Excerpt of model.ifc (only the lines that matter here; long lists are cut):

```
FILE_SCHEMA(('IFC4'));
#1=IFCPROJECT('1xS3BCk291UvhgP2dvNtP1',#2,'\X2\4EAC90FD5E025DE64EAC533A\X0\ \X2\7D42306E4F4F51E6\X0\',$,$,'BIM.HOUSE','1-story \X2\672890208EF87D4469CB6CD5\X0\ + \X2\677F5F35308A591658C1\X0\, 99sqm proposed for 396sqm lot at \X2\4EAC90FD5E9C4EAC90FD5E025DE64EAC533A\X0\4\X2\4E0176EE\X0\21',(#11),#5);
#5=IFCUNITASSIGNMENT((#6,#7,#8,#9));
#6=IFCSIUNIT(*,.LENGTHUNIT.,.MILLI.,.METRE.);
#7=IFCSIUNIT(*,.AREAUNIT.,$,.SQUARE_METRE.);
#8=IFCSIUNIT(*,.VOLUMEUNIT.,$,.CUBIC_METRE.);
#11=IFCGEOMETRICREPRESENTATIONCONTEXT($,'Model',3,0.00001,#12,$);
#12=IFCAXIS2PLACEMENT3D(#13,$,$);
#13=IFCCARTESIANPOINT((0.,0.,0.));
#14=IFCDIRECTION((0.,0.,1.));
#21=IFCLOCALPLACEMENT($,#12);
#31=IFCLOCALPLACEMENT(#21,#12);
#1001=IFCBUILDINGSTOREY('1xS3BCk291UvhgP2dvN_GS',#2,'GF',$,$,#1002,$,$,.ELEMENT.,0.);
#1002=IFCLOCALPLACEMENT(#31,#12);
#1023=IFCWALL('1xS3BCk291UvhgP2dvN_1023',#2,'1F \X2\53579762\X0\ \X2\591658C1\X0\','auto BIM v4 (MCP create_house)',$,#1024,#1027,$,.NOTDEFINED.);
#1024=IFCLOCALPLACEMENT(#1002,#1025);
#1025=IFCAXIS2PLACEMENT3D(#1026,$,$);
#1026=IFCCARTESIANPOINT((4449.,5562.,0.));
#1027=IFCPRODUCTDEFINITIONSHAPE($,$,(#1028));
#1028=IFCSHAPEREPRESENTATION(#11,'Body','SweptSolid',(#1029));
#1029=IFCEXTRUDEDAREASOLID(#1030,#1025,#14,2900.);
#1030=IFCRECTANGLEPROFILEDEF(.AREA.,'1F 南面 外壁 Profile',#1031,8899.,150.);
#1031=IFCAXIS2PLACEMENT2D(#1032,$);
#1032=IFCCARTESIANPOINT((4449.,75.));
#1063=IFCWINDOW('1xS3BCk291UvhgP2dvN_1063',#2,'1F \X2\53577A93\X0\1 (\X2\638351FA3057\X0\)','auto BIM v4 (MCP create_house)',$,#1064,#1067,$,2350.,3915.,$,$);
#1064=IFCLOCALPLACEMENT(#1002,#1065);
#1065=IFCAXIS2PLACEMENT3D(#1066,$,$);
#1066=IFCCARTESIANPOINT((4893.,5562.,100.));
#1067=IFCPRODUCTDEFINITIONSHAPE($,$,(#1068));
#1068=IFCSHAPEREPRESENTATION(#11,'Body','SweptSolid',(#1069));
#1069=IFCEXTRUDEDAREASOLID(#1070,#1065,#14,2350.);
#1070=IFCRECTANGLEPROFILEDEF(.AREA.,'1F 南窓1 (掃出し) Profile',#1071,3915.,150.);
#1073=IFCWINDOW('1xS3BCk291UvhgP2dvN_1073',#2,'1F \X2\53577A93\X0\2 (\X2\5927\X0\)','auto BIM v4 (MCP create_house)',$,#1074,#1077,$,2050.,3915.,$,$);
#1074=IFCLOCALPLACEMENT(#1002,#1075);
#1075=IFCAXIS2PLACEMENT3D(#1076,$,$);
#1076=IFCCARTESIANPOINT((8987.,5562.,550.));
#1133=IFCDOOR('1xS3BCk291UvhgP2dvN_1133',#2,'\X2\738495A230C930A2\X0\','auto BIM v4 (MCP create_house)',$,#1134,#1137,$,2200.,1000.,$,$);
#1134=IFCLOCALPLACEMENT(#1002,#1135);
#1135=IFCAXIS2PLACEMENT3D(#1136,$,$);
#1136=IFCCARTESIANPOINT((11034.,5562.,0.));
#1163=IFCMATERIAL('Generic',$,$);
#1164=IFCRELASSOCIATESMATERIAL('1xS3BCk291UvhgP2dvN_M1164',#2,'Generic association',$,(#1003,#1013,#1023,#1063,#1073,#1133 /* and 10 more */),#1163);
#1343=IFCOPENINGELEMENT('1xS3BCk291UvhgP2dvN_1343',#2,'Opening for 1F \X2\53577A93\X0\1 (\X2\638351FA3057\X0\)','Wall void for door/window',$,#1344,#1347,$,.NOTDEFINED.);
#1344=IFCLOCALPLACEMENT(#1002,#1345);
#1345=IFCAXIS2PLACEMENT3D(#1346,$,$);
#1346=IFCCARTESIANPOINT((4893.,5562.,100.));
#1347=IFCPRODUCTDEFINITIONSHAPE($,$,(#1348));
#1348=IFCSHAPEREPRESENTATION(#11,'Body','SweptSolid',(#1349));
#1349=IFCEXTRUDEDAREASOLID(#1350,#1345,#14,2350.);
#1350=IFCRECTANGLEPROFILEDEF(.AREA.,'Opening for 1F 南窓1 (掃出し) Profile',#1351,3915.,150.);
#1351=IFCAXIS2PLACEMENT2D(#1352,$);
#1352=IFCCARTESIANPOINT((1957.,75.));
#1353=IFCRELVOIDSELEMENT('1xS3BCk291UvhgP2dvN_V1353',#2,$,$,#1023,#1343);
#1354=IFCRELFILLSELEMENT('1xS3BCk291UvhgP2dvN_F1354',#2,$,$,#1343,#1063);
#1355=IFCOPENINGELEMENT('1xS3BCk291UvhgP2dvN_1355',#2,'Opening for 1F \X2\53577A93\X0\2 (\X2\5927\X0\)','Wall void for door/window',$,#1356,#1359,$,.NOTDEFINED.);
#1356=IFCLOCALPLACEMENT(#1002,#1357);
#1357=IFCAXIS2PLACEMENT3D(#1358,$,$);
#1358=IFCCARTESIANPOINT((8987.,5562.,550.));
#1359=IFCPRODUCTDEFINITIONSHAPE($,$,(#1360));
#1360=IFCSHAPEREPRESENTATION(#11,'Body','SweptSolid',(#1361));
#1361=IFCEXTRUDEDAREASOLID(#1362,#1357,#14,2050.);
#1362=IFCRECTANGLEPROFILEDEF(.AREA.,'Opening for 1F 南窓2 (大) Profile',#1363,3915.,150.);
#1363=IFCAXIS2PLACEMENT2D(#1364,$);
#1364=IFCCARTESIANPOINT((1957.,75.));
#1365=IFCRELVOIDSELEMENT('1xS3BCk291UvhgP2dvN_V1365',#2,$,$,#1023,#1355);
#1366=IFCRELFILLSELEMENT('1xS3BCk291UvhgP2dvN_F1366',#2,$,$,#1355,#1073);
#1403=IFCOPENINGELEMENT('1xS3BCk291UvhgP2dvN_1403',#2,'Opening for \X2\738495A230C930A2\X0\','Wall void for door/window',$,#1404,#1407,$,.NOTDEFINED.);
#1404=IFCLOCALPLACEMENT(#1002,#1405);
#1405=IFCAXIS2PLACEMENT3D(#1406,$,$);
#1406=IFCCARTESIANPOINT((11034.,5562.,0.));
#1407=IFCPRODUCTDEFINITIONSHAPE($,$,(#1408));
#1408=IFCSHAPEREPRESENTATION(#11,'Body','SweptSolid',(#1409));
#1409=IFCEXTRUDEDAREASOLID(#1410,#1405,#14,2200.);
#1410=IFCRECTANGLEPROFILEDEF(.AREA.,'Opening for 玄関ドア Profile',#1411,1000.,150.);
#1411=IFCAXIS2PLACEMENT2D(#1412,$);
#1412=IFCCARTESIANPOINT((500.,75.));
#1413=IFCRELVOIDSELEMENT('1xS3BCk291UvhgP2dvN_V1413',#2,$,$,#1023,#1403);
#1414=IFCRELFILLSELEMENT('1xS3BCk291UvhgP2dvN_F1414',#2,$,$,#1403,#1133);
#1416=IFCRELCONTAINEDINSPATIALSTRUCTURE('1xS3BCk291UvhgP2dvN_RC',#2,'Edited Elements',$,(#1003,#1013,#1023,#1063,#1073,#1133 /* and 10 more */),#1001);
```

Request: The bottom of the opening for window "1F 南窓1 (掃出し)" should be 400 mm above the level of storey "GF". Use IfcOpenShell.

```python
import numpy as np
import ifcopenshell
import ifcopenshell.api.geometry
import ifcopenshell.geom
import ifcopenshell.util.element
import ifcopenshell.util.placement
import ifcopenshell.util.shape
import ifcopenshell.util.unit

model = ifcopenshell.open("model.ifc")
unit_scale = ifcopenshell.util.unit.calculate_unit_scale(model)

window = model.by_guid("1xS3BCk291UvhgP2dvN_1063")
opening = window.FillsVoids[0].RelatingOpeningElement
storey = ifcopenshell.util.element.get_container(window, ifc_class="IfcBuildingStorey")
level = ifcopenshell.util.placement.get_local_placement(storey.ObjectPlacement)[2, 3]

# The opening's origin need not be at the sill, so measure its lowest point.
shape = ifcopenshell.geom.create_shape(ifcopenshell.geom.settings(), opening)
bottom = ifcopenshell.util.shape.get_shape_bottom_elevation(shape, shape.geometry) / unit_scale
dz = level + 400.0 - bottom

shift = np.array([0.0, 0.0, dz])
# The window is not placed relative to its opening, so move both.
for product in (opening, window):
    matrix = ifcopenshell.util.placement.get_local_placement(product.ObjectPlacement)
    matrix[:3, 3] += shift
    ifcopenshell.api.geometry.edit_object_placement(model, product=product, matrix=matrix, is_si=False)

print(f"moved by {dz * unit_scale:+.3f} m")

model.write("model_v2.ifc")
```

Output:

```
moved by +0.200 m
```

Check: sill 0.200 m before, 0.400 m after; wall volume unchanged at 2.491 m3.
